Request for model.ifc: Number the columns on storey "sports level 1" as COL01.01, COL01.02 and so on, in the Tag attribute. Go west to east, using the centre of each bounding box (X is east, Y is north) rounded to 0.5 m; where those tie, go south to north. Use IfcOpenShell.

First a look at what the model holds.

```python
import ifcopenshell
import ifcopenshell.util.element
import ifcopenshell.util.placement

model = ifcopenshell.open("model.ifc")
print(model.schema)
storey = next(s for s in model.by_type("IfcBuildingStorey") if s.Name == "sports level 1")
columns = [e for e in ifcopenshell.util.element.get_decomposition(storey) if e.is_a("IfcColumn")]
for e in sorted(columns, key=lambda e: e.id()):
    origin = ifcopenshell.util.placement.get_local_placement(e.ObjectPlacement)[:3, 3]
    print(e.id(), e.Tag, e.Name, origin.round(2) + 0.0, sep=" | ")
```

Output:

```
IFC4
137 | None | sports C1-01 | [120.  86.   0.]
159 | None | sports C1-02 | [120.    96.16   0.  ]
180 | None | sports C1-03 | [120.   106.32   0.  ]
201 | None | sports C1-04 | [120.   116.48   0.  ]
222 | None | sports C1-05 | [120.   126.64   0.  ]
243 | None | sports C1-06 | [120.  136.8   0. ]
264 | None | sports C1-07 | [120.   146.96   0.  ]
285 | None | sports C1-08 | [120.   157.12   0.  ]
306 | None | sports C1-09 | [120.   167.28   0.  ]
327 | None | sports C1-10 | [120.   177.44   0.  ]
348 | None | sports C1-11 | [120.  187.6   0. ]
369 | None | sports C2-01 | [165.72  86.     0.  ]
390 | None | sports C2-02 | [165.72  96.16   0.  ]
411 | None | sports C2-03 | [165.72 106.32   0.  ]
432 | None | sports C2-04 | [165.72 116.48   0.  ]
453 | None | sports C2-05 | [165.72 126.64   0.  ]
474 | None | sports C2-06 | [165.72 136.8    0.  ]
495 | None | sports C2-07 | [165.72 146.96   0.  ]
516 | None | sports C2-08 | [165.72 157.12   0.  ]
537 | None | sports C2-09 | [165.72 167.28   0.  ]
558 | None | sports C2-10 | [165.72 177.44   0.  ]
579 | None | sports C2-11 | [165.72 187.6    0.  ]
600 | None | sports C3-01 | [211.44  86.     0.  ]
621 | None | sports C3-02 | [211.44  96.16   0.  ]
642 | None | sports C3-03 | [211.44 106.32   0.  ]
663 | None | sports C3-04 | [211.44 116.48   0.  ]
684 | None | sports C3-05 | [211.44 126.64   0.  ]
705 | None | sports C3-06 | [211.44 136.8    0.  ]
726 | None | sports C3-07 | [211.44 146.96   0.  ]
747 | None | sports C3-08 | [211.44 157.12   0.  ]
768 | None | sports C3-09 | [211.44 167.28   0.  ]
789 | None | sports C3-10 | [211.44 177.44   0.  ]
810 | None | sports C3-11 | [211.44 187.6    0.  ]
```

```python
import ifcopenshell
import ifcopenshell.geom
import ifcopenshell.util.element
import ifcopenshell.util.shape

model = ifcopenshell.open("model.ifc")
settings = ifcopenshell.geom.settings()
settings.set("use-world-coords", True)


def centre(element):
    shape = ifcopenshell.geom.create_shape(settings, element)
    return ifcopenshell.util.shape.get_bbox_centroid(shape.geometry)


storey = next(s for s in model.by_type("IfcBuildingStorey") if s.Name == "sports level 1")
columns = [e for e in ifcopenshell.util.element.get_decomposition(storey) if e.is_a("IfcColumn")]

# Insertion points can sit at a corner or the storey origin, so sort by the geometry (in metres).
centres = {e: centre(e) for e in columns}
columns.sort(key=lambda e: (round(centres[e][0] / 0.5), centres[e][1]))

for i, e in enumerate(columns, start=1):
    number = f"COL01.{i:02d}"
    e.Tag = number
    print(e.id(), number)

model.write("model_v2.ifc")
```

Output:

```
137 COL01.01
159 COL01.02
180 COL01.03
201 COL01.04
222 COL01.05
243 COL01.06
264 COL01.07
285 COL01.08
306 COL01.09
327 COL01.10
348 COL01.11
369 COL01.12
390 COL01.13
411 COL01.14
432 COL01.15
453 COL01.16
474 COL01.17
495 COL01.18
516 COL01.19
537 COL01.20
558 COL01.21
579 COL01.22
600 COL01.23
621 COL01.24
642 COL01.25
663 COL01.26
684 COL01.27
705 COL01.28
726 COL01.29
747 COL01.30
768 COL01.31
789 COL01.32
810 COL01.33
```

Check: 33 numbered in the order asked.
